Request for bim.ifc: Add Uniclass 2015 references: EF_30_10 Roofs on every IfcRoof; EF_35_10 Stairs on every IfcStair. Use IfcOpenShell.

First a look at what the model holds.

```python
import ifcopenshell

model = ifcopenshell.open("bim.ifc")
print(model.schema)
print("classifications:", [c.Name for c in model.by_type("IfcClassification")])
for ifc_class in ("IfcDoor", "IfcRoof", "IfcStair", "IfcWall", "IfcWindow"):
    print(ifc_class, len(model.by_type(ifc_class)))
```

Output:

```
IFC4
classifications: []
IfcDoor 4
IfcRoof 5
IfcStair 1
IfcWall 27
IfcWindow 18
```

```python
import ifcopenshell
import ifcopenshell.api.classification

model = ifcopenshell.open("bim.ifc")

system = ifcopenshell.api.classification.add_classification(model, classification="Uniclass 2015")

codes = {
    "IfcRoof": ("EF_30_10", "Roofs"),
    "IfcStair": ("EF_35_10", "Stairs"),
}
for ifc_class, (code, name) in codes.items():
    products = model.by_type(ifc_class)
    ifcopenshell.api.classification.add_reference(
        model, products=products, classification=system, identification=code, name=name
    )
    print(code, len(products))

model.write("bim_updated.ifc")
```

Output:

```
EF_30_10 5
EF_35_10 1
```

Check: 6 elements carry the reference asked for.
